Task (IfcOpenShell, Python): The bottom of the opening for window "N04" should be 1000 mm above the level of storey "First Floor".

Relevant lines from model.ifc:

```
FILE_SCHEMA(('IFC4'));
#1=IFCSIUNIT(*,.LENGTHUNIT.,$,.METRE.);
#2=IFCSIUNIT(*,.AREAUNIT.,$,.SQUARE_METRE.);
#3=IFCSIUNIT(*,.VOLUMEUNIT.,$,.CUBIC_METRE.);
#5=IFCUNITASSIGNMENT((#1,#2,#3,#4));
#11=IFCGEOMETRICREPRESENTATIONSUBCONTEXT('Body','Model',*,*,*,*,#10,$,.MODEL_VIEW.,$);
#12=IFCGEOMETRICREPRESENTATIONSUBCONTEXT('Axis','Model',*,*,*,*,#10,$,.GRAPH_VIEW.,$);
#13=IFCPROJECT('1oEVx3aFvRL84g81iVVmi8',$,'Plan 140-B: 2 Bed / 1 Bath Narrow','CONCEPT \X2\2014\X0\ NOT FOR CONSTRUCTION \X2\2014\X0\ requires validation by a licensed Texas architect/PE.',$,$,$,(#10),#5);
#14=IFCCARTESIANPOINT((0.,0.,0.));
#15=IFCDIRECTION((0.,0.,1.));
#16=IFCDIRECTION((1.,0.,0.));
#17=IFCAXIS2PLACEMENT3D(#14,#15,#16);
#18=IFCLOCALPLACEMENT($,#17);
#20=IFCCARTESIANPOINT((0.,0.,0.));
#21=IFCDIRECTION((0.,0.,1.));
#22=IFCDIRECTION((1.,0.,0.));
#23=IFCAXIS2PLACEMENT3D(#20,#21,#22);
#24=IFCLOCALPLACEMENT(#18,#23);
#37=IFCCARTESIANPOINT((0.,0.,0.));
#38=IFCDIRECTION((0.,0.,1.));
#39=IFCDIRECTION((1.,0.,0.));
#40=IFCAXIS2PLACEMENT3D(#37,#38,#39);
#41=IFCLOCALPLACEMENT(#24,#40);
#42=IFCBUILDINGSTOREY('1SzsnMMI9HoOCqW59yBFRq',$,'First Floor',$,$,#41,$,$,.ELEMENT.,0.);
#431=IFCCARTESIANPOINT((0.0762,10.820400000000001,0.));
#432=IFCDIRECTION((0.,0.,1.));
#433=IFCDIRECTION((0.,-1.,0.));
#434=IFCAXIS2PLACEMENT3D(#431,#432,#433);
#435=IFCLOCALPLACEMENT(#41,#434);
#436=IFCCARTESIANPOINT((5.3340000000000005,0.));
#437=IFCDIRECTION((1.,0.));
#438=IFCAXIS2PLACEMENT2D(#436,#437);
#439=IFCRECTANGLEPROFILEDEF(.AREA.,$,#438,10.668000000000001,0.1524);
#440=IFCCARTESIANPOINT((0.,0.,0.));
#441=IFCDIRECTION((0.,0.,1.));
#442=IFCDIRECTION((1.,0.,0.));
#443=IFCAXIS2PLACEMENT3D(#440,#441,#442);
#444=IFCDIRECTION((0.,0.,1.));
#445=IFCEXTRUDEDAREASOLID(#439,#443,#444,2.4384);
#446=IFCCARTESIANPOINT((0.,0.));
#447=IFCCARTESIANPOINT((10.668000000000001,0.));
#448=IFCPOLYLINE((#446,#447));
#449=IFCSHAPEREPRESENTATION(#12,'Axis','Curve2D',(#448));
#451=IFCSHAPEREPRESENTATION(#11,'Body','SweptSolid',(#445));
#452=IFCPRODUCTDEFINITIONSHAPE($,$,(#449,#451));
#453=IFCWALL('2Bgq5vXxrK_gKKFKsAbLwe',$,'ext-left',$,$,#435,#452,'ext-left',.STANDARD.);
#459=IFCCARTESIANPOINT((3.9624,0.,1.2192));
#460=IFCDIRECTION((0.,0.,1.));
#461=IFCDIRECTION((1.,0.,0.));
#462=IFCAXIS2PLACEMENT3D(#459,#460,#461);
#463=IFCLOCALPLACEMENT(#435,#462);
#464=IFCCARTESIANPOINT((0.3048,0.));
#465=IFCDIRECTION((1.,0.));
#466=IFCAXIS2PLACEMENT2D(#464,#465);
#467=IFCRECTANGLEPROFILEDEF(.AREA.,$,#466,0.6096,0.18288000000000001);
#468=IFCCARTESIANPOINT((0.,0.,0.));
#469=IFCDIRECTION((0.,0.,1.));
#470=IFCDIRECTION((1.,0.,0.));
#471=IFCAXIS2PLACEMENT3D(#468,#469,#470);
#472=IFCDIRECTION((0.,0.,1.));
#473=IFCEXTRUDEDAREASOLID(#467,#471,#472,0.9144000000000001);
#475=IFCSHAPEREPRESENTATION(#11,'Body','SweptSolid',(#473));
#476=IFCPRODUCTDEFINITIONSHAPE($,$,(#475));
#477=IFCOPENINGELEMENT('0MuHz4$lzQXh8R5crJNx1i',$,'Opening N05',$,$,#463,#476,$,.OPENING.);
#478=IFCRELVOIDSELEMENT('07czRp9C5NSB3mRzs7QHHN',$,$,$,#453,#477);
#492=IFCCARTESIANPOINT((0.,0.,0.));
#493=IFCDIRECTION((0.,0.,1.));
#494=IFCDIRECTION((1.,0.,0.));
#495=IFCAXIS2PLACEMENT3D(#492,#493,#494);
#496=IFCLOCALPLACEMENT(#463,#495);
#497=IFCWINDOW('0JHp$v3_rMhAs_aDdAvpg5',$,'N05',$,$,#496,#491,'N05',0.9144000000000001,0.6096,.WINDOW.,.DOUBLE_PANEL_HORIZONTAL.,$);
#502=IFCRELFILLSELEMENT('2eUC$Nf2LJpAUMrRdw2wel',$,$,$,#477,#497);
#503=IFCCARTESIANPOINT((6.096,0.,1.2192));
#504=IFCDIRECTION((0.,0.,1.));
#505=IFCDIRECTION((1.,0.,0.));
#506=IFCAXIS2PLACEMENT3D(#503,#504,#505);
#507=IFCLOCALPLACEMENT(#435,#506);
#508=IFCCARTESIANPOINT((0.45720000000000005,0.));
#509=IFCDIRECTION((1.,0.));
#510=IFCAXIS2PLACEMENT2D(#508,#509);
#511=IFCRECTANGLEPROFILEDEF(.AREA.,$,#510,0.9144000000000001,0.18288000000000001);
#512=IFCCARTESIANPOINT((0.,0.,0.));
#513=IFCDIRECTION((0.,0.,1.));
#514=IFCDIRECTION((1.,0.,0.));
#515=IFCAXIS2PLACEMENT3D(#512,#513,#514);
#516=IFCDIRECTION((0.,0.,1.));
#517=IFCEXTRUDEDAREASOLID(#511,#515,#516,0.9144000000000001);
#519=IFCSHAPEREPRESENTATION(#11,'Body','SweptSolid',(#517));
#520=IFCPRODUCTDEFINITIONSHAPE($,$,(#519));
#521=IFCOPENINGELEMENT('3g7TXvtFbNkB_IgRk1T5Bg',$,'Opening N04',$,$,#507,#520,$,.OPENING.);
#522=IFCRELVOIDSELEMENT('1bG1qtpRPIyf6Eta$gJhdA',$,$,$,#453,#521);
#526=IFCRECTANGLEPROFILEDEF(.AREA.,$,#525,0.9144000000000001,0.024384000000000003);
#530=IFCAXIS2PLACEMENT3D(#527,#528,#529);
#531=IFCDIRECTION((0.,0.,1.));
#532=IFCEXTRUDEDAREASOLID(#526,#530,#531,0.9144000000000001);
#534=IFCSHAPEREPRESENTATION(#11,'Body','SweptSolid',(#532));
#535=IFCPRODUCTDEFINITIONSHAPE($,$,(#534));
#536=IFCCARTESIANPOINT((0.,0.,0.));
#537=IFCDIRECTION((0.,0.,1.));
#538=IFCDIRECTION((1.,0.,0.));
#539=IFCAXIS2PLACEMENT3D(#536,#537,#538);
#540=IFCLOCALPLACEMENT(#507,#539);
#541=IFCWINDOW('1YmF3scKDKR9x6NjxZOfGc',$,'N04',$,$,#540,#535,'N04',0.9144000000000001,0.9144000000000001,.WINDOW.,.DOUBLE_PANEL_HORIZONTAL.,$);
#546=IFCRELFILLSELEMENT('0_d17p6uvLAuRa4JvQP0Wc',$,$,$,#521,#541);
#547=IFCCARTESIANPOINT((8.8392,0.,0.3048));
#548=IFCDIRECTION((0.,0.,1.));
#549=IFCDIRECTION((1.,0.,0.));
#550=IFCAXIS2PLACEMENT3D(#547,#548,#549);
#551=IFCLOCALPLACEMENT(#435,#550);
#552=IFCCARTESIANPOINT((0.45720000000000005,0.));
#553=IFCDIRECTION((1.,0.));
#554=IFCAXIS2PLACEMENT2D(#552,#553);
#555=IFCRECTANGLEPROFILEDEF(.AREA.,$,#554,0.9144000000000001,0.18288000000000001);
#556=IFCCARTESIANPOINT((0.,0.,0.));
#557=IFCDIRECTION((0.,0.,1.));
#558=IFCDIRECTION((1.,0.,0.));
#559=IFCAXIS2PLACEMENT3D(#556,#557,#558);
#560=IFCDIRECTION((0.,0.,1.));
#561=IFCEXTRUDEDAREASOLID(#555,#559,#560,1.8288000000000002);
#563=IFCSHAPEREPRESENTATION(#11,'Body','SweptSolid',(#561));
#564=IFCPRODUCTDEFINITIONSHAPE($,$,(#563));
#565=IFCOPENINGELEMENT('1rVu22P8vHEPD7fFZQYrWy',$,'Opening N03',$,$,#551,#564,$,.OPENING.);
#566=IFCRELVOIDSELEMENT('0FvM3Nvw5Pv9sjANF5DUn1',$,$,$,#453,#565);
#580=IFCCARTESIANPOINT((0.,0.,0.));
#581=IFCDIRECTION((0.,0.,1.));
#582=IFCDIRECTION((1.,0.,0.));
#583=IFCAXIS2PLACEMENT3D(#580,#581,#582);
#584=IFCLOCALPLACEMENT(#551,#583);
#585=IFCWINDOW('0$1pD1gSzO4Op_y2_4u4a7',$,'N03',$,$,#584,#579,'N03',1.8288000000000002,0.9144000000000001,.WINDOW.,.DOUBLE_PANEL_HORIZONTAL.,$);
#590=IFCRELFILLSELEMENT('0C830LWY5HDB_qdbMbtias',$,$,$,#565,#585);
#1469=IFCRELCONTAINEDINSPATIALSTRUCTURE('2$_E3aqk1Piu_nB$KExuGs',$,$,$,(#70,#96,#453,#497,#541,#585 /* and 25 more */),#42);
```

```python
import numpy as np
import ifcopenshell
import ifcopenshell.api.geometry
import ifcopenshell.geom
import ifcopenshell.util.element
import ifcopenshell.util.placement
import ifcopenshell.util.shape
import ifcopenshell.util.unit

model = ifcopenshell.open("model.ifc")
unit_scale = ifcopenshell.util.unit.calculate_unit_scale(model)

window = model.by_guid("1YmF3scKDKR9x6NjxZOfGc")
opening = window.FillsVoids[0].RelatingOpeningElement
storey = ifcopenshell.util.element.get_container(window, ifc_class="IfcBuildingStorey")
level = ifcopenshell.util.placement.get_local_placement(storey.ObjectPlacement)[2, 3]

# The opening's origin need not be at the sill, so measure its lowest point.
shape = ifcopenshell.geom.create_shape(ifcopenshell.geom.settings(), opening)
bottom = ifcopenshell.util.shape.get_shape_bottom_elevation(shape, shape.geometry) / unit_scale
dz = level + 1.0 - bottom

shift = np.array([0.0, 0.0, dz])
# The window is placed relative to its opening, so it follows when the opening moves.
matrix = ifcopenshell.util.placement.get_local_placement(opening.ObjectPlacement)
matrix[:3, 3] += shift
ifcopenshell.api.geometry.edit_object_placement(
    model, product=opening, matrix=matrix, is_si=False, should_transform_children=True
)

print(f"moved by {dz * unit_scale:+.3f} m")

model.write("model_updated.ifc")
```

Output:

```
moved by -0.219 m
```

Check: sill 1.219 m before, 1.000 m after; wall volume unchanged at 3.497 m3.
